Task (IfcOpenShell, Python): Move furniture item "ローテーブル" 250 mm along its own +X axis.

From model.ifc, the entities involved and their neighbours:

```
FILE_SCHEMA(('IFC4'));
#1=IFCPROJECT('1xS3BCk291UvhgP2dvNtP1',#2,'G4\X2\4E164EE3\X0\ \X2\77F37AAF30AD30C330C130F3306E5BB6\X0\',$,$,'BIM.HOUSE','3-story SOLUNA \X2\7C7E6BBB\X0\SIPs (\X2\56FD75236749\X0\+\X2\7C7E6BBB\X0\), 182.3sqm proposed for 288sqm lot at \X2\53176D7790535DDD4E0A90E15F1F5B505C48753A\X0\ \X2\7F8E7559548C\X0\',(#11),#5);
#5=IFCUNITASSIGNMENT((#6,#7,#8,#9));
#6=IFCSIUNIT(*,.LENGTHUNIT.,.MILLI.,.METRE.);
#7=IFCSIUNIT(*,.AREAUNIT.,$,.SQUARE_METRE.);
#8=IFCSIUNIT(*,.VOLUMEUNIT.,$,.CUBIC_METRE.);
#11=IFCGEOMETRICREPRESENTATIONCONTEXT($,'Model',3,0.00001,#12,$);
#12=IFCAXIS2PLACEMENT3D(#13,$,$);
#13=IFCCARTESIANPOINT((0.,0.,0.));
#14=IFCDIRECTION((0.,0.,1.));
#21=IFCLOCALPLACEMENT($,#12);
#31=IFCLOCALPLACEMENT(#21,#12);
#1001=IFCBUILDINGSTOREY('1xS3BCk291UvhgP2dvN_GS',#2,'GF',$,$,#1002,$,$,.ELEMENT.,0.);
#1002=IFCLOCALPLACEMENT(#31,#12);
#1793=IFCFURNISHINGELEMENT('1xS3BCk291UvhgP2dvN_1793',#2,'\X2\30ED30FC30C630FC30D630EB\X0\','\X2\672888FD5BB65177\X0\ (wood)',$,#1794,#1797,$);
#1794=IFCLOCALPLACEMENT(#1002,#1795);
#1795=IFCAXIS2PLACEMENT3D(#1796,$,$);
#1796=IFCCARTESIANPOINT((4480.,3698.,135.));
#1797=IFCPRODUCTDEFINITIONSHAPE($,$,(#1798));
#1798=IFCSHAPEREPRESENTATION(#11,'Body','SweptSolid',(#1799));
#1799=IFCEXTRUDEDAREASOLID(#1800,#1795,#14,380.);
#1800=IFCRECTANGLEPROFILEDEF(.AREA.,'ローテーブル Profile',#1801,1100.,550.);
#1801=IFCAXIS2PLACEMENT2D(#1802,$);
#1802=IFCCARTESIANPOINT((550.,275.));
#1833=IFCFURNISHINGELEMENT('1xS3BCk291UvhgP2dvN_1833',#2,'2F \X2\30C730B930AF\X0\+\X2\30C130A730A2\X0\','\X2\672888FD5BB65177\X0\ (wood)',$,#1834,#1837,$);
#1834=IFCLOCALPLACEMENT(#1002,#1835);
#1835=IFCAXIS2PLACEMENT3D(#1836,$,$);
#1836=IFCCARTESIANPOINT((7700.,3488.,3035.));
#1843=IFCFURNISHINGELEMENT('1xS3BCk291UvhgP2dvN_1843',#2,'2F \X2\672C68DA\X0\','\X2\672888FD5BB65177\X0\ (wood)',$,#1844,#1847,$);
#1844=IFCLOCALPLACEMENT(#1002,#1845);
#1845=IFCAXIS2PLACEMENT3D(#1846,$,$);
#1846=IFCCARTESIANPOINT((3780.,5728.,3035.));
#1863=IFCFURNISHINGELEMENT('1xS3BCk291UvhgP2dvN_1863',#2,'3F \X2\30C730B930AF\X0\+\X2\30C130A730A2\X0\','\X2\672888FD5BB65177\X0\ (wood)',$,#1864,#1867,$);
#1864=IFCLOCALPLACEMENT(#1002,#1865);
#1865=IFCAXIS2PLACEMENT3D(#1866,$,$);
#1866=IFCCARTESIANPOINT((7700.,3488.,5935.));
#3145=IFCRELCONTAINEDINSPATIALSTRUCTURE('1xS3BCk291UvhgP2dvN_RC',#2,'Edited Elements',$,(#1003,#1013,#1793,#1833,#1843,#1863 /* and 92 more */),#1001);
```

```python
import ifcopenshell
import ifcopenshell.api.geometry
import ifcopenshell.util.placement
import ifcopenshell.util.unit

model = ifcopenshell.open("model.ifc")
unit_scale = ifcopenshell.util.unit.calculate_unit_scale(model)

item = model.by_guid("1xS3BCk291UvhgP2dvN_1793")
matrix = ifcopenshell.util.placement.get_local_placement(item.ObjectPlacement)
matrix[:3, 3] += matrix[:3, 0] * 0.25 / unit_scale
ifcopenshell.api.geometry.edit_object_placement(model, product=item, matrix=matrix, is_si=False)

print(ifcopenshell.util.placement.get_local_placement(item.ObjectPlacement).round(3) + 0.0)

model.write("model_rev.ifc")
```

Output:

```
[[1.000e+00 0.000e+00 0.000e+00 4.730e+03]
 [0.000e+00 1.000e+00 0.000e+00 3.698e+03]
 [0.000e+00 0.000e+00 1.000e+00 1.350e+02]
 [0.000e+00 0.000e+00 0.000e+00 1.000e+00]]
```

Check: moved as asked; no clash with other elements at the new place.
